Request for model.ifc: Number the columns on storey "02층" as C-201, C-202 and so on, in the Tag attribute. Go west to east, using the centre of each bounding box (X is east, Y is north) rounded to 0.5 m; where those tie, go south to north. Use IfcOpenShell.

First a look at what the model holds.

```python
import ifcopenshell
import ifcopenshell.util.element
import ifcopenshell.util.placement

model = ifcopenshell.open("model.ifc")
print(model.schema)
storey = next(s for s in model.by_type("IfcBuildingStorey") if s.Name == "02층")
columns = [e for e in ifcopenshell.util.element.get_decomposition(storey) if e.is_a("IfcColumn")]
for e in sorted(columns, key=lambda e: e.id()):
    origin = ifcopenshell.util.placement.get_local_placement(e.ObjectPlacement)[:3, 3]
    print(e.id(), e.Tag, e.Name, origin.round(2) + 0.0, sep=" | ")
```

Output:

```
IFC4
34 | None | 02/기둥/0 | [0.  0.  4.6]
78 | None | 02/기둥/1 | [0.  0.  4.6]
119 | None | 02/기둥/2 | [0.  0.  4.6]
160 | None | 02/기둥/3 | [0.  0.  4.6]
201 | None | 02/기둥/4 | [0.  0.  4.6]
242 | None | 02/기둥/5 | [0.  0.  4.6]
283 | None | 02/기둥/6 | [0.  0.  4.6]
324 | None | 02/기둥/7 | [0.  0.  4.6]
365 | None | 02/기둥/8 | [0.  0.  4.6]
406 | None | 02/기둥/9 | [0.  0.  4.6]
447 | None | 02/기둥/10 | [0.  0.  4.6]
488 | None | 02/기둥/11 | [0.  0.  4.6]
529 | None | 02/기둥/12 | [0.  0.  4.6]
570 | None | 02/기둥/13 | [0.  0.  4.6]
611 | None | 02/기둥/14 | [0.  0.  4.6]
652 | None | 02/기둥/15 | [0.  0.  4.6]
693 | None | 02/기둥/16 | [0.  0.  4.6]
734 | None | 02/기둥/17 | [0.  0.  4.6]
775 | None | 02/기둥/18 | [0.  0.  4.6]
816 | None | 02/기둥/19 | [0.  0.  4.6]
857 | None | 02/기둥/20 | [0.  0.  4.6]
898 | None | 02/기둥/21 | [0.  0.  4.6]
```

```python
import ifcopenshell
import ifcopenshell.geom
import ifcopenshell.util.element
import ifcopenshell.util.shape

model = ifcopenshell.open("model.ifc")
settings = ifcopenshell.geom.settings()
settings.set("use-world-coords", True)


def centre(element):
    shape = ifcopenshell.geom.create_shape(settings, element)
    return ifcopenshell.util.shape.get_bbox_centroid(shape.geometry)


storey = next(s for s in model.by_type("IfcBuildingStorey") if s.Name == "02층")
columns = [e for e in ifcopenshell.util.element.get_decomposition(storey) if e.is_a("IfcColumn")]

# Insertion points can sit at a corner or the storey origin, so sort by the geometry (in metres).
centres = {e: centre(e) for e in columns}
columns.sort(key=lambda e: (round(centres[e][0] / 0.5), centres[e][1]))

for i, e in enumerate(columns, start=1):
    number = f"C-2{i:02d}"
    e.Tag = number
    print(e.id(), number)

model.write("model_updated.ifc")
```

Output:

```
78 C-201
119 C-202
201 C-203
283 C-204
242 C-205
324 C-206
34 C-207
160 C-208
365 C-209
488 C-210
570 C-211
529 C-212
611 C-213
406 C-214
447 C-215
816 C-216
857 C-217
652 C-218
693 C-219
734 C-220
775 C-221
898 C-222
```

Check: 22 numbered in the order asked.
